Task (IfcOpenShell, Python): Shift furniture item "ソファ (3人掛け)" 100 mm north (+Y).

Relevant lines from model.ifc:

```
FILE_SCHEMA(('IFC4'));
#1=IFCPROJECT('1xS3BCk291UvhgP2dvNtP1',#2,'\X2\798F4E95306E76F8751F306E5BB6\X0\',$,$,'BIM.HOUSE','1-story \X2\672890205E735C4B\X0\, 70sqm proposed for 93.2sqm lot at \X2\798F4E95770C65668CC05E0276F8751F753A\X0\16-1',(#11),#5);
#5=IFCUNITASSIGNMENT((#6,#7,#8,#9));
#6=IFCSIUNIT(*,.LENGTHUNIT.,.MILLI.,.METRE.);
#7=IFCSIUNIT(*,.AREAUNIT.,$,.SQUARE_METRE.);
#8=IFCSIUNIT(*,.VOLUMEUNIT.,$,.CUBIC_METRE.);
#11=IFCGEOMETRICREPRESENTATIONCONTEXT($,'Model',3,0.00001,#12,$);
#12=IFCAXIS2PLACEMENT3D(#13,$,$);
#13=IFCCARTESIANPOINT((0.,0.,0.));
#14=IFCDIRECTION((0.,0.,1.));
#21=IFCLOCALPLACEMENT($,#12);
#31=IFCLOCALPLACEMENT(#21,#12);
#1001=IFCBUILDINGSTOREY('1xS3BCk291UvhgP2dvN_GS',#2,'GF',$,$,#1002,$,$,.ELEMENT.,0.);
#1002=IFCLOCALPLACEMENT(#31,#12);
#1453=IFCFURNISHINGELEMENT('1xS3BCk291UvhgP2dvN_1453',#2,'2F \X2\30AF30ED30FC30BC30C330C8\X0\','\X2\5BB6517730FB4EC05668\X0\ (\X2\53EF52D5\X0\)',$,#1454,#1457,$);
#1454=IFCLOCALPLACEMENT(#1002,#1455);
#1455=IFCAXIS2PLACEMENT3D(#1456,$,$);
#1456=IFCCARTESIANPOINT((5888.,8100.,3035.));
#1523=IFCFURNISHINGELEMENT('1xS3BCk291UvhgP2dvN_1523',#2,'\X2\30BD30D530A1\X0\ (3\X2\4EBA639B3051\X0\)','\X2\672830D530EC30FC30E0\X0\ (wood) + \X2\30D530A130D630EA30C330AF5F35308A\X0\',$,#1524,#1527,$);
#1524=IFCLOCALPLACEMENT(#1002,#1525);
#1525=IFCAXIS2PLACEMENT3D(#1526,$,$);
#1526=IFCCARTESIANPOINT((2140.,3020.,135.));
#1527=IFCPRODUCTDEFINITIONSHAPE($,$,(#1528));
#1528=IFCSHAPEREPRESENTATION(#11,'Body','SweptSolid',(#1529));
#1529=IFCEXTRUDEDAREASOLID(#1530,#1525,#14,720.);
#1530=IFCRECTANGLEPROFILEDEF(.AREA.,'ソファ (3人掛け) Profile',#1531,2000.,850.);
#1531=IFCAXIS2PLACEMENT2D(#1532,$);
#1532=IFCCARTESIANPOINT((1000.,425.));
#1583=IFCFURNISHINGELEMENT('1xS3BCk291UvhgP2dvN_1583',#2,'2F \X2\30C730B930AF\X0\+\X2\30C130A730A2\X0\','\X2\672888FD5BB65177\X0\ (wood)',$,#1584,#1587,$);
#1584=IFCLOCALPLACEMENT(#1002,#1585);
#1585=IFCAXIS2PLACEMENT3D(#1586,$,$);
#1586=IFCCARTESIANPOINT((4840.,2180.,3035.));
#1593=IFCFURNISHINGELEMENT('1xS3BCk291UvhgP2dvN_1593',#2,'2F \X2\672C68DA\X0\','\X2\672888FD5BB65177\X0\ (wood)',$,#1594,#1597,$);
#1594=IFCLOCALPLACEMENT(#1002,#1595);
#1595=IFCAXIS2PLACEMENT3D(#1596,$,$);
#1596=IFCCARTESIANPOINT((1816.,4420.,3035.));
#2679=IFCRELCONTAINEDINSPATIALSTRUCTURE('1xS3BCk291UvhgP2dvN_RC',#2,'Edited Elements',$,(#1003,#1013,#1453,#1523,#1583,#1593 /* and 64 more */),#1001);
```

```python
import ifcopenshell
import ifcopenshell.api.geometry
import ifcopenshell.util.placement
import ifcopenshell.util.unit

model = ifcopenshell.open("model.ifc")
unit_scale = ifcopenshell.util.unit.calculate_unit_scale(model)

item = model.by_guid("1xS3BCk291UvhgP2dvN_1523")
matrix = ifcopenshell.util.placement.get_local_placement(item.ObjectPlacement)
matrix[1, 3] += 0.1 / unit_scale
ifcopenshell.api.geometry.edit_object_placement(model, product=item, matrix=matrix, is_si=False)

print(ifcopenshell.util.placement.get_local_placement(item.ObjectPlacement).round(3) + 0.0)

model.write("model_edited.ifc")
```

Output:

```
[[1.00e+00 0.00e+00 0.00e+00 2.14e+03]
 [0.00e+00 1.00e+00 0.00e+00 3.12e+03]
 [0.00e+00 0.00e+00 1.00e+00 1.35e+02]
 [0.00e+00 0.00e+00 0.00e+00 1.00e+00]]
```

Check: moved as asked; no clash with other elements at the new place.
